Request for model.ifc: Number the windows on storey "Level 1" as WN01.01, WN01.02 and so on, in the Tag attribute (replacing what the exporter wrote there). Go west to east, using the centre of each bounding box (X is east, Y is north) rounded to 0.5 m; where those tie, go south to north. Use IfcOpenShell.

First a look at what the model holds.

```python
import ifcopenshell
import ifcopenshell.util.element
import ifcopenshell.util.placement

model = ifcopenshell.open("model.ifc")
print(model.schema)
storey = next(s for s in model.by_type("IfcBuildingStorey") if s.Name == "Level 1")
windows = [e for e in ifcopenshell.util.element.get_decomposition(storey) if e.is_a("IfcWindow")]
for e in sorted(windows, key=lambda e: e.id()):
    origin = ifcopenshell.util.placement.get_local_placement(e.ObjectPlacement)[:3, 3]
    print(e.id(), e.Tag, e.Name, origin.round(2) + 0.0, sep=" | ")
```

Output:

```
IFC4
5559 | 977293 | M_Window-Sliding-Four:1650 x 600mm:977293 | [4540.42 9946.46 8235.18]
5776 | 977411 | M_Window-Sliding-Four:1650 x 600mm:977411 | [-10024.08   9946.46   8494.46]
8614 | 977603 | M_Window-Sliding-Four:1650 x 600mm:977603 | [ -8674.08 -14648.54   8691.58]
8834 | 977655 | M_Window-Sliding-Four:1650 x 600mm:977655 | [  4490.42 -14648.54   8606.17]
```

```python
import ifcopenshell
import ifcopenshell.geom
import ifcopenshell.util.element
import ifcopenshell.util.shape

model = ifcopenshell.open("model.ifc")
settings = ifcopenshell.geom.settings()
settings.set("use-world-coords", True)


def centre(element):
    shape = ifcopenshell.geom.create_shape(settings, element)
    return ifcopenshell.util.shape.get_bbox_centroid(shape.geometry)


storey = next(s for s in model.by_type("IfcBuildingStorey") if s.Name == "Level 1")
windows = [e for e in ifcopenshell.util.element.get_decomposition(storey) if e.is_a("IfcWindow")]

# Insertion points can sit at a corner or the storey origin, so sort by the geometry (in metres).
centres = {e: centre(e) for e in windows}
windows.sort(key=lambda e: (round(centres[e][0] / 0.5), centres[e][1]))

for i, e in enumerate(windows, start=1):
    number = f"WN01.{i:02d}"
    e.Tag = number
    print(e.id(), number)

model.write("model_edited.ifc")
```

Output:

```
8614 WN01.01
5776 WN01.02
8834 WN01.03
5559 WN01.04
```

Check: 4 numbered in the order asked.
